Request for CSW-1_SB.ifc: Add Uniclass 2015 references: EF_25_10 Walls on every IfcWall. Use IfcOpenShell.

First a look at what the model holds.

```python
import ifcopenshell

model = ifcopenshell.open("CSW-1_SB.ifc")
print(model.schema)
print("classifications:", [c.Name for c in model.by_type("IfcClassification")])
for ifc_class in ("IfcDoor", "IfcRoof", "IfcStair", "IfcWall", "IfcWindow"):
    print(ifc_class, len(model.by_type(ifc_class)))
```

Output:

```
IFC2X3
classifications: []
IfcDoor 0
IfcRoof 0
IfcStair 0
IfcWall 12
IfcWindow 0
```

```python
import ifcopenshell
import ifcopenshell.api.classification

model = ifcopenshell.open("CSW-1_SB.ifc")

# IFC2X3 requires Source and Edition and has no link from the project to the system.
system = model.create_entity("IfcClassification", Source="NBS", Edition="2015", Name="Uniclass 2015")

codes = {
    "IfcWall": ("EF_25_10", "Walls"),
}
for ifc_class, (code, name) in codes.items():
    products = model.by_type(ifc_class)
    ifcopenshell.api.classification.add_reference(
        model, products=products, classification=system, identification=code, name=name
    )
    print(code, len(products))

model.write("CSW-1_SB_edited.ifc")
```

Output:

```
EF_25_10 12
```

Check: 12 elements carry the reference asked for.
